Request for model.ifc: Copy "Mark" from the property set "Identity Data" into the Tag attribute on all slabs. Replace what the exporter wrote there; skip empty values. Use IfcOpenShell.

First a look at what the model holds.

```python
import ifcopenshell
import ifcopenshell.util.element

model = ifcopenshell.open("model.ifc")
print(model.schema)
slabs = model.by_type("IfcSlab")
print(len(slabs), "slabs")
for e in slabs[:8]:
    source = ifcopenshell.util.element.get_pset(e, "Identity Data", "Mark")
    target = e.Tag
    print(e.id(), repr(source), repr(target), sep=" | ")
```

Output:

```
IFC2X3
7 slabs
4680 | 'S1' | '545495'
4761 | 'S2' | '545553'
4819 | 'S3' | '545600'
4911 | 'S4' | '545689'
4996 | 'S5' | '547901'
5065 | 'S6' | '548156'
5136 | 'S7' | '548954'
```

```python
import ifcopenshell
import ifcopenshell.util.element

model = ifcopenshell.open("model.ifc")

count = 0
for e in model.by_type("IfcSlab"):
    value = ifcopenshell.util.element.get_pset(e, "Identity Data", "Mark")
    current = e.Tag
    if not value or not value.strip() or current == value:
        continue
    e.Tag = value
    count += 1

print(count, "slabs updated")

model.write("model_rev.ifc")
```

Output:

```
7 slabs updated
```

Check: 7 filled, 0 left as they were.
